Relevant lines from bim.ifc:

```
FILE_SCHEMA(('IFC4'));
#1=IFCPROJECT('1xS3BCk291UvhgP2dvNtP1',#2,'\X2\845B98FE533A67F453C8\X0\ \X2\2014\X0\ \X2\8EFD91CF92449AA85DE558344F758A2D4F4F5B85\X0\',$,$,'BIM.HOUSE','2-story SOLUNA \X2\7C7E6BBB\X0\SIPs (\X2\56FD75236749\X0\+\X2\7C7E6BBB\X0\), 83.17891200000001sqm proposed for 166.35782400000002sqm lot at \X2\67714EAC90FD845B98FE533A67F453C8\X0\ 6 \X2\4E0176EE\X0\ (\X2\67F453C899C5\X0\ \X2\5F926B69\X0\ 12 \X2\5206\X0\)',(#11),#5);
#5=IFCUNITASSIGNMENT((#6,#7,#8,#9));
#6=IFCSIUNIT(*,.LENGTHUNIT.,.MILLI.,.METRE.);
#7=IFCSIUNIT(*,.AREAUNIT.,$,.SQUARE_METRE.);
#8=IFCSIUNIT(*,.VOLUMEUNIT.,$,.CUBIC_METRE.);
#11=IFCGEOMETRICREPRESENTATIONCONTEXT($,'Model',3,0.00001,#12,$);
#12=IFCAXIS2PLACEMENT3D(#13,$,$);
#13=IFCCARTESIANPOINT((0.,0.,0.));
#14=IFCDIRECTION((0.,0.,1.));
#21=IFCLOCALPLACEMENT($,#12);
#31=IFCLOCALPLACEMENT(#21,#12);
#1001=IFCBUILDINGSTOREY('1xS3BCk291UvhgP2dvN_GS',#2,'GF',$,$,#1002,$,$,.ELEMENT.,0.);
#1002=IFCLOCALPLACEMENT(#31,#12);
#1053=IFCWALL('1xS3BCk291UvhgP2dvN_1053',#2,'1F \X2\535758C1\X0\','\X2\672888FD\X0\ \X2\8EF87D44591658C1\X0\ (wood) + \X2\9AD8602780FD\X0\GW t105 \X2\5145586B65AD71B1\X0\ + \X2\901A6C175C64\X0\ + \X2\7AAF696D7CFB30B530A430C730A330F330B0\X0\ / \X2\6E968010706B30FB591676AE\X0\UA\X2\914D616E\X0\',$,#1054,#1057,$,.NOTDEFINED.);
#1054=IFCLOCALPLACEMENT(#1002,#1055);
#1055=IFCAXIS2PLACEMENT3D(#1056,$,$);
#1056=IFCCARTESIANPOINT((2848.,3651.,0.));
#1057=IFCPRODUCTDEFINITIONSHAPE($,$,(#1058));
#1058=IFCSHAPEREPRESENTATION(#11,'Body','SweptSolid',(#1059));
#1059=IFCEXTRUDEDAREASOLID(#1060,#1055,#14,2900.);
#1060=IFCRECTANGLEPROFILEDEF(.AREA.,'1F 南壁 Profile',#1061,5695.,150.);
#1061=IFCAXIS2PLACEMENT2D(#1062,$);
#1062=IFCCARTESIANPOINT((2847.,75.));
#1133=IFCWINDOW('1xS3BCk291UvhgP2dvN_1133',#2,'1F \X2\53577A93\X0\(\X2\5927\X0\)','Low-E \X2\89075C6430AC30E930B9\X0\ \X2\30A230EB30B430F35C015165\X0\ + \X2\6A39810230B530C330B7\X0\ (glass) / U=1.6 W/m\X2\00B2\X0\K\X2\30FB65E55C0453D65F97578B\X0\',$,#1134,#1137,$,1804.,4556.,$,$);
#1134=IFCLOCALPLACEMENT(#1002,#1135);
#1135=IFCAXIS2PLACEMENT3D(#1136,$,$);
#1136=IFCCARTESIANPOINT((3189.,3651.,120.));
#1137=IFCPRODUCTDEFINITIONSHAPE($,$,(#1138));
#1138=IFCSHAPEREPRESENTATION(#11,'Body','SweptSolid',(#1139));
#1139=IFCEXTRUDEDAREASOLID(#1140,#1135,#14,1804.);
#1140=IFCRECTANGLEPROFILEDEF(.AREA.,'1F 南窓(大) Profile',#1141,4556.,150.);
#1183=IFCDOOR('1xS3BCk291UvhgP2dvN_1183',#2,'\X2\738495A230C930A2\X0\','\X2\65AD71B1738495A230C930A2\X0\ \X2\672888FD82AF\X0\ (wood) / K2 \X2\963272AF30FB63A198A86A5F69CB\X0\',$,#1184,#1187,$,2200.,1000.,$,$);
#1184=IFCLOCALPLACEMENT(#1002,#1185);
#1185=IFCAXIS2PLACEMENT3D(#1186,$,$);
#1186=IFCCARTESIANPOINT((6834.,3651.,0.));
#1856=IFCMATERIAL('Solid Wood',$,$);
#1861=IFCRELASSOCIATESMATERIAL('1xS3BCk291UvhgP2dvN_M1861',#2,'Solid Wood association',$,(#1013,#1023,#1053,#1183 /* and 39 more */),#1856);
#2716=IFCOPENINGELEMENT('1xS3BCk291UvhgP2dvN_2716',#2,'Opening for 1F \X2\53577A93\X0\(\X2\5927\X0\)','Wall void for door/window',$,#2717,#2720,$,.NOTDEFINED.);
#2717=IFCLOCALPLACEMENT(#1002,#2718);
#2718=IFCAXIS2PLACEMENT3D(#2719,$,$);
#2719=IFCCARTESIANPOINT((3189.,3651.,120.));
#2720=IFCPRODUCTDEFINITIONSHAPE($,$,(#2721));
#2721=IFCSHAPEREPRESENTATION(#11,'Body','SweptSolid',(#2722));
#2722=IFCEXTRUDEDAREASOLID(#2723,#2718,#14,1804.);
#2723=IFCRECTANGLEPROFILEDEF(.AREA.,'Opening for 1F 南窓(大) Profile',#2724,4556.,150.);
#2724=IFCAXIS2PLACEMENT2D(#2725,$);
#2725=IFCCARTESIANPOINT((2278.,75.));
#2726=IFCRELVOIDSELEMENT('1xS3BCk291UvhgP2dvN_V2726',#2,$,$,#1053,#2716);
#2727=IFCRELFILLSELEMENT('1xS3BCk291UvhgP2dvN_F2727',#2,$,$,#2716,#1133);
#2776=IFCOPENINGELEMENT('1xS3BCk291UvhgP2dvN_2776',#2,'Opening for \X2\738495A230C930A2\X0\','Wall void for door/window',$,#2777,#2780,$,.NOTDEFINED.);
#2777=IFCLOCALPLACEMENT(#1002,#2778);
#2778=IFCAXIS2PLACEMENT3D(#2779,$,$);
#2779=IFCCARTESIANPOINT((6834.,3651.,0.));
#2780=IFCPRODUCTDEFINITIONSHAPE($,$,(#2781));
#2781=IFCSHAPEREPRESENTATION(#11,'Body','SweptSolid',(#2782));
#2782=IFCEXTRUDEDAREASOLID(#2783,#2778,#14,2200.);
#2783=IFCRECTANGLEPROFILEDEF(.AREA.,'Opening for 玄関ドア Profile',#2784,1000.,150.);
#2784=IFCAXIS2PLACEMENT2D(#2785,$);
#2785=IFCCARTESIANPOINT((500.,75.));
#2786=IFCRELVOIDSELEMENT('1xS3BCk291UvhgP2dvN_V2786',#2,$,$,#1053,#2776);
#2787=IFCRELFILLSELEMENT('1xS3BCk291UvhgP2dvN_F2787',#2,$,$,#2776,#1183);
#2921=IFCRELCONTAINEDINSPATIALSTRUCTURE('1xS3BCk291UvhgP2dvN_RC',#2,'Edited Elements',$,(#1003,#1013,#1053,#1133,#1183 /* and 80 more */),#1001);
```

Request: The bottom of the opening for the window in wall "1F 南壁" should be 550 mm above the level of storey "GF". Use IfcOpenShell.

```python
import numpy as np
import ifcopenshell
import ifcopenshell.api.geometry
import ifcopenshell.geom
import ifcopenshell.util.element
import ifcopenshell.util.placement
import ifcopenshell.util.shape
import ifcopenshell.util.unit

model = ifcopenshell.open("bim.ifc")
unit_scale = ifcopenshell.util.unit.calculate_unit_scale(model)

window = model.by_guid("1xS3BCk291UvhgP2dvN_1133")
opening = window.FillsVoids[0].RelatingOpeningElement
storey = ifcopenshell.util.element.get_container(window, ifc_class="IfcBuildingStorey")
level = ifcopenshell.util.placement.get_local_placement(storey.ObjectPlacement)[2, 3]

# The opening's origin need not be at the sill, so measure its lowest point.
shape = ifcopenshell.geom.create_shape(ifcopenshell.geom.settings(), opening)
bottom = ifcopenshell.util.shape.get_shape_bottom_elevation(shape, shape.geometry) / unit_scale
dz = level + 0.55 / unit_scale - bottom

shift = np.array([0.0, 0.0, dz])
# The window is not placed relative to its opening, so move both.
for product in (opening, window):
    matrix = ifcopenshell.util.placement.get_local_placement(product.ObjectPlacement)
    matrix[:3, 3] += shift
    ifcopenshell.api.geometry.edit_object_placement(model, product=product, matrix=matrix, is_si=False)

print(f"moved by {dz * unit_scale:+.3f} m")

model.write("bim_rev.ifc")
```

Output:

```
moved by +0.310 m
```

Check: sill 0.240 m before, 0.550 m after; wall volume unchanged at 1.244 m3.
